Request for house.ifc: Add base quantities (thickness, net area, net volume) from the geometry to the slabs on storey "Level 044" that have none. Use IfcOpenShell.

First a look at what the model holds.

```python
import ifcopenshell
import ifcopenshell.util.element
import ifcopenshell.util.unit

model = ifcopenshell.open("house.ifc")
print(model.schema)
for unit_type in ("LENGTHUNIT", "AREAUNIT", "VOLUMEUNIT"):
    print(unit_type, ifcopenshell.util.unit.calculate_unit_scale(model, unit_type))
storey = next(s for s in model.by_type("IfcBuildingStorey") if s.Name == "Level 044")
slabs = [e for e in ifcopenshell.util.element.get_decomposition(storey) if e.is_a("IfcSlab")]
for e in sorted(slabs, key=lambda e: e.id()):
    print(e.id(), e.is_a(), e.Name, list(ifcopenshell.util.element.get_psets(e, qtos_only=True)), sep=" | ")
```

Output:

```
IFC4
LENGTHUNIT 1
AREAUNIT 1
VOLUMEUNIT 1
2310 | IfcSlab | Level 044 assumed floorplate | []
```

```python
import ifcopenshell
import ifcopenshell.api.pset
import ifcopenshell.geom
import ifcopenshell.util.element
import ifcopenshell.util.shape
import ifcopenshell.util.unit

model = ifcopenshell.open("house.ifc")
unit_scale = ifcopenshell.util.unit.calculate_unit_scale(model)
area_scale = ifcopenshell.util.unit.calculate_unit_scale(model, "AREAUNIT")
volume_scale = ifcopenshell.util.unit.calculate_unit_scale(model, "VOLUMEUNIT")
settings = ifcopenshell.geom.settings()

storey = next(s for s in model.by_type("IfcBuildingStorey") if s.Name == "Level 044")
slabs = [e for e in ifcopenshell.util.element.get_decomposition(storey) if e.is_a("IfcSlab")]

for e in sorted(slabs, key=lambda e: e.id()):
    if ifcopenshell.util.element.get_psets(e, qtos_only=True, should_inherit=False):
        continue
    # Geometry comes back in metres, in the element's own axes.
    shape = ifcopenshell.geom.create_shape(settings, e)
    values = {
        "Width": ifcopenshell.util.shape.get_z(shape.geometry) / unit_scale,
        "NetArea": ifcopenshell.util.shape.get_footprint_area(shape.geometry) / area_scale,
        "NetVolume": ifcopenshell.util.shape.get_volume(shape.geometry) / volume_scale,
    }
    qto = ifcopenshell.api.pset.add_qto(model, product=e, name="Qto_SlabBaseQuantities")
    ifcopenshell.api.pset.edit_qto(model, qto=qto, properties=values)
    print(e.id(), {k: round(v, 3) for k, v in values.items()})

model.write("house_edited.ifc")
```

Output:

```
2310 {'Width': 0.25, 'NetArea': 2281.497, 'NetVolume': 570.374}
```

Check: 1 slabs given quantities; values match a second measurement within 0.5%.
